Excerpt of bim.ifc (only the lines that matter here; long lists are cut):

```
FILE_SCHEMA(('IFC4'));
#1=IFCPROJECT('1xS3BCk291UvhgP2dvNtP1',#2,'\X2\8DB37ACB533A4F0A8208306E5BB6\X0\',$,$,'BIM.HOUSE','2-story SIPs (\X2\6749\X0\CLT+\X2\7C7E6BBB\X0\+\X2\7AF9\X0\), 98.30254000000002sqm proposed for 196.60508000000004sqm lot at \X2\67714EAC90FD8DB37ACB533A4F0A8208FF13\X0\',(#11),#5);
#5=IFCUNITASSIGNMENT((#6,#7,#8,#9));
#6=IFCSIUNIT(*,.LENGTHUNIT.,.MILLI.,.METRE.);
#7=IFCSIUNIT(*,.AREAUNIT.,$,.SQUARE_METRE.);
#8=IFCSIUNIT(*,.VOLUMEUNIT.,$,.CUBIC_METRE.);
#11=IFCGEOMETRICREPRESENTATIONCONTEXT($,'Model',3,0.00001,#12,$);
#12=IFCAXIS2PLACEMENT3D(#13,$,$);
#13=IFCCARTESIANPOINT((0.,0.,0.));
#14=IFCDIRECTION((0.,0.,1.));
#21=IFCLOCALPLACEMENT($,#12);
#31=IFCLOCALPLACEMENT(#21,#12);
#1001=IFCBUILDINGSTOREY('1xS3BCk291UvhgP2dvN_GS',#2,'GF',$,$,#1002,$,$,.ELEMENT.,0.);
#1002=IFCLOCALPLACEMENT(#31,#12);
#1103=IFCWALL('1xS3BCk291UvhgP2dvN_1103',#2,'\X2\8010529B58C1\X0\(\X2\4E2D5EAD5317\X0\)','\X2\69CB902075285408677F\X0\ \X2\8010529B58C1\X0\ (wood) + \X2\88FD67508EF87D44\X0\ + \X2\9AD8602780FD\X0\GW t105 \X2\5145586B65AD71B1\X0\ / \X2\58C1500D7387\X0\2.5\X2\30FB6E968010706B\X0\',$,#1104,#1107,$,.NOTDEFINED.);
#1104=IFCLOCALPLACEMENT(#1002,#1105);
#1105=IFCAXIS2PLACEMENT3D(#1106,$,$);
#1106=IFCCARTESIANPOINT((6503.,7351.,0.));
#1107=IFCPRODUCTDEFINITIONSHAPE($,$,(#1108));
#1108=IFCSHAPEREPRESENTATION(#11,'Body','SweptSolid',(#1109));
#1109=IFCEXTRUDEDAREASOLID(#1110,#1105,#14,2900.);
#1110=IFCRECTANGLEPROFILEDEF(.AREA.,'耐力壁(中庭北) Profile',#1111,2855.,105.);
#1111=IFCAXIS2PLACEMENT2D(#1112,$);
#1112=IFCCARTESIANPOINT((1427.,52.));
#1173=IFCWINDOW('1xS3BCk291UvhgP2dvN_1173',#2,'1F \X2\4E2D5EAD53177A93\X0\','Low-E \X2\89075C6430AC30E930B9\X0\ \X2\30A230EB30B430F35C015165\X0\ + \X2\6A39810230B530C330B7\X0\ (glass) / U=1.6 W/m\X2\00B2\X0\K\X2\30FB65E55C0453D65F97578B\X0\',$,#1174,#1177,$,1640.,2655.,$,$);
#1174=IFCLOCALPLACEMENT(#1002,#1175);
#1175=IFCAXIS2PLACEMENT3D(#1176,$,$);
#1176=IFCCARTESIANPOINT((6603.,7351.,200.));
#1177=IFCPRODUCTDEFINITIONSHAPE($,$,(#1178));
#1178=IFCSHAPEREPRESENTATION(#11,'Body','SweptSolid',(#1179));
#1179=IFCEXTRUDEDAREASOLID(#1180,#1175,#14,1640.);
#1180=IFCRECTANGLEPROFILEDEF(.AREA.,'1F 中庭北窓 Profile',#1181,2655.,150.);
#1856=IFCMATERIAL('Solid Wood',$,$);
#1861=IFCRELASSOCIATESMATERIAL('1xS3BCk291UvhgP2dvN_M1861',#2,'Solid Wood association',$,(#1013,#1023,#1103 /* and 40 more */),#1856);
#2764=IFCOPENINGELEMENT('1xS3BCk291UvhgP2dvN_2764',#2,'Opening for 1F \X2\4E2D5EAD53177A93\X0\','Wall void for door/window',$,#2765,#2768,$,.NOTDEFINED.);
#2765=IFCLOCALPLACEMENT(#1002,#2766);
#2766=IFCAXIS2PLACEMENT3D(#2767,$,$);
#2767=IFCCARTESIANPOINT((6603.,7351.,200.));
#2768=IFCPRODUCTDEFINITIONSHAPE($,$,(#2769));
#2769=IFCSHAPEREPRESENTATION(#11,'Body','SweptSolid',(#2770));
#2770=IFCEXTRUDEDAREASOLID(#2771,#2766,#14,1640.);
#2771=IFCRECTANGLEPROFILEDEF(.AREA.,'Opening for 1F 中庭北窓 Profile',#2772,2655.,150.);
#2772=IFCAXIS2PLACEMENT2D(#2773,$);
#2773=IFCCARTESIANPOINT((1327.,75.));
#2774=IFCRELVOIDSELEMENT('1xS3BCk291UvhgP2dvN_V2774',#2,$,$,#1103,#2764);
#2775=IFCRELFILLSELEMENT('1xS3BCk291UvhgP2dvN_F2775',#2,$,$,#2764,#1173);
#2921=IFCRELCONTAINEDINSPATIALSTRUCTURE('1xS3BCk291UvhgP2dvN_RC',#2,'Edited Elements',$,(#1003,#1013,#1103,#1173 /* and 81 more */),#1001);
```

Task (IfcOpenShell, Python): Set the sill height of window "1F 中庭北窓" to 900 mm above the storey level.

```python
import numpy as np
import ifcopenshell
import ifcopenshell.api.geometry
import ifcopenshell.geom
import ifcopenshell.util.element
import ifcopenshell.util.placement
import ifcopenshell.util.shape
import ifcopenshell.util.unit

model = ifcopenshell.open("bim.ifc")
unit_scale = ifcopenshell.util.unit.calculate_unit_scale(model)

window = model.by_id(1173)
opening = window.FillsVoids[0].RelatingOpeningElement
storey = ifcopenshell.util.element.get_container(window, ifc_class="IfcBuildingStorey")
level = ifcopenshell.util.placement.get_local_placement(storey.ObjectPlacement)[2, 3]

# The opening's origin need not be at the sill, so measure its lowest point.
shape = ifcopenshell.geom.create_shape(ifcopenshell.geom.settings(), opening)
bottom = ifcopenshell.util.shape.get_shape_bottom_elevation(shape, shape.geometry) / unit_scale
dz = level + 900.0 - bottom

shift = np.array([0.0, 0.0, dz])
# The window is not placed relative to its opening, so move both.
for product in (opening, window):
    matrix = ifcopenshell.util.placement.get_local_placement(product.ObjectPlacement)
    matrix[:3, 3] += shift
    ifcopenshell.api.geometry.edit_object_placement(model, product=product, matrix=matrix, is_si=False)

print(f"moved by {dz * unit_scale:+.3f} m")

model.write("bim_updated.ifc")
```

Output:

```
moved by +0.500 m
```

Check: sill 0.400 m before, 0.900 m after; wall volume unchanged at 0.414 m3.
